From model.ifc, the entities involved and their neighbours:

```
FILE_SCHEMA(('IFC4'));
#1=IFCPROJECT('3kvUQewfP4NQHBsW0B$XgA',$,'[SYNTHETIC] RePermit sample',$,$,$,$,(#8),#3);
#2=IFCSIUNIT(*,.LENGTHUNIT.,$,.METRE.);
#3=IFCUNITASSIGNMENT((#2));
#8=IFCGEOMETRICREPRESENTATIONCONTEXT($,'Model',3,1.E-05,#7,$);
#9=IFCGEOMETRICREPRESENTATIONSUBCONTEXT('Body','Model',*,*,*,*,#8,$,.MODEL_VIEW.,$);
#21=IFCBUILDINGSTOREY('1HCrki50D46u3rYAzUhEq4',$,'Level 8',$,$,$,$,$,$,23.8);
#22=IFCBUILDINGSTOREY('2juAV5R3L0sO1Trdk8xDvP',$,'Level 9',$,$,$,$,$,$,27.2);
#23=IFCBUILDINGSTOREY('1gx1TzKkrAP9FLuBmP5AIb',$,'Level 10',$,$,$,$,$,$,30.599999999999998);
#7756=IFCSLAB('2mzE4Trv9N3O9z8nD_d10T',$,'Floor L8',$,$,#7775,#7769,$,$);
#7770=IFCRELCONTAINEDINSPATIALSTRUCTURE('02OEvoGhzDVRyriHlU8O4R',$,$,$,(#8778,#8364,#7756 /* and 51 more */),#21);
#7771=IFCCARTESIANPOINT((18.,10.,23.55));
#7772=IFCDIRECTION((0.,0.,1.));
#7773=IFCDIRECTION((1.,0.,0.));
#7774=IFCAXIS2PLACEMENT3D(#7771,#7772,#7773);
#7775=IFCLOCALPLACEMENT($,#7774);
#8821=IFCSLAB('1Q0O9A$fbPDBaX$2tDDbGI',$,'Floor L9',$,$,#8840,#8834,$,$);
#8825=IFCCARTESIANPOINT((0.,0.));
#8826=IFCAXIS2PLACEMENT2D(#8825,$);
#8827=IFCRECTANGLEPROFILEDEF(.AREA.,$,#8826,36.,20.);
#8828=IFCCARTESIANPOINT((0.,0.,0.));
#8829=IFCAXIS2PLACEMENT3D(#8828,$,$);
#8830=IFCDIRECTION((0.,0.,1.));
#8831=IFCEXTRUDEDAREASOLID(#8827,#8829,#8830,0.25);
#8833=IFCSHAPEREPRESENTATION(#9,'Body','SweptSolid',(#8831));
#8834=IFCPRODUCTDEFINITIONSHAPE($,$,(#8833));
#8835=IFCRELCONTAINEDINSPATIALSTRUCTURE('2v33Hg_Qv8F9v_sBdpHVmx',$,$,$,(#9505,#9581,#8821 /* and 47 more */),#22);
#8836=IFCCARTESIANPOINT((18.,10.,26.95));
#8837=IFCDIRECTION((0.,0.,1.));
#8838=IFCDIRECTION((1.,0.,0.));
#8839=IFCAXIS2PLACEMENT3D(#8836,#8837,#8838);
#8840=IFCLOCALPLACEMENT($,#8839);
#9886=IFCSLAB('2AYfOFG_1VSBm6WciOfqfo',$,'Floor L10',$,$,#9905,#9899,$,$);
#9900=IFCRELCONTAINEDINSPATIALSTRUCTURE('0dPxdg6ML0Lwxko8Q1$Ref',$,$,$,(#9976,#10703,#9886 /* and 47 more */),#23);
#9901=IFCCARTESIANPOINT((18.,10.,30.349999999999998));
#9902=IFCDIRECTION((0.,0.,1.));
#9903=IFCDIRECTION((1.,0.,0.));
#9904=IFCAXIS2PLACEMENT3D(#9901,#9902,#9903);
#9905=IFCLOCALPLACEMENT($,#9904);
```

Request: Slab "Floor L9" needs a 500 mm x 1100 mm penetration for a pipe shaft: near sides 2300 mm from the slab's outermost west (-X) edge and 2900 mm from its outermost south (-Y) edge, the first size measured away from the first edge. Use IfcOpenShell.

```python
import numpy as np
import ifcopenshell
import ifcopenshell.api.feature
import ifcopenshell.api.geometry
import ifcopenshell.api.root
import ifcopenshell.geom
import ifcopenshell.util.placement
import ifcopenshell.util.representation
import ifcopenshell.util.shape
import ifcopenshell.util.unit

model = ifcopenshell.open("model.ifc")
unit_scale = ifcopenshell.util.unit.calculate_unit_scale(model)
settings = ifcopenshell.geom.settings()


def volume(element):
    """Net volume in cubic metres, openings subtracted."""
    shape = ifcopenshell.geom.create_shape(settings, element)
    return ifcopenshell.util.shape.get_volume(shape.geometry)


slab = model.by_guid("1Q0O9A$fbPDBaX$2tDDbGI")
before = volume(slab)

# Extent in the slab's own axes, in metres. The edges named are its -X and -Y sides.
slab_shape = ifcopenshell.geom.create_shape(settings, slab)
vertices = ifcopenshell.util.shape.get_vertices(slab_shape.geometry)
x_min, y_min, bottom = vertices.min(axis=0)
top = vertices[:, 2].max()

opening = ifcopenshell.api.root.create_entity(model, ifc_class="IfcOpeningElement", name="Pipe shaft opening", predefined_type="OPENING")
context = ifcopenshell.util.representation.get_context(model, "Model", "Body", "MODEL_VIEW")
width, depth = 0.5, 1.1
outline = [(0.0, 0.0), (width, 0.0), (width, depth), (0.0, depth), (0.0, 0.0)]
# Overshoot both faces by 50 mm so the cut is clean.
shape = ifcopenshell.api.geometry.add_slab_representation(
    model, context=context, depth=top - bottom + 0.1, polyline=outline
)
ifcopenshell.api.geometry.assign_representation(model, product=opening, representation=shape)

matrix = ifcopenshell.util.placement.get_local_placement(slab.ObjectPlacement)
matrix[:, 3] = matrix @ np.append(np.array([x_min + 2.3, y_min + 2.9, bottom - 0.05]) / unit_scale, 1.0)
ifcopenshell.api.geometry.edit_object_placement(model, product=opening, matrix=matrix, is_si=False)
ifcopenshell.api.feature.add_feature(model, feature=opening, element=slab)

after = volume(slab)

print(f"slab volume {before:.3f} -> {after:.3f} m3")

model.write("model-out.ifc")
```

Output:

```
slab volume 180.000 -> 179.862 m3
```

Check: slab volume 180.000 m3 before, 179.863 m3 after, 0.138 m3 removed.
